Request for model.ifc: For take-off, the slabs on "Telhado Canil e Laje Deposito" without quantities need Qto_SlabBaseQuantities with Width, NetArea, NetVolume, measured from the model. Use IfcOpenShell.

First a look at what the model holds.

```python
import ifcopenshell
import ifcopenshell.util.element
import ifcopenshell.util.unit

model = ifcopenshell.open("model.ifc")
print(model.schema)
for unit_type in ("LENGTHUNIT", "AREAUNIT", "VOLUMEUNIT"):
    print(unit_type, ifcopenshell.util.unit.calculate_unit_scale(model, unit_type))
storey = next(s for s in model.by_type("IfcBuildingStorey") if s.Name == "Telhado Canil e Laje Deposito")
slabs = [e for e in ifcopenshell.util.element.get_decomposition(storey) if e.is_a("IfcSlab")]
for e in sorted(slabs, key=lambda e: e.id()):
    print(e.id(), e.is_a(), e.Name, list(ifcopenshell.util.element.get_psets(e, qtos_only=True)), sep=" | ")
```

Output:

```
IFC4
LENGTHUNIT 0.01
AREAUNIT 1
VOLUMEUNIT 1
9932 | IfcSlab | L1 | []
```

```python
import ifcopenshell
import ifcopenshell.api.pset
import ifcopenshell.geom
import ifcopenshell.util.element
import ifcopenshell.util.shape
import ifcopenshell.util.unit

model = ifcopenshell.open("model.ifc")
unit_scale = ifcopenshell.util.unit.calculate_unit_scale(model)
area_scale = ifcopenshell.util.unit.calculate_unit_scale(model, "AREAUNIT")
volume_scale = ifcopenshell.util.unit.calculate_unit_scale(model, "VOLUMEUNIT")
settings = ifcopenshell.geom.settings()

storey = next(s for s in model.by_type("IfcBuildingStorey") if s.Name == "Telhado Canil e Laje Deposito")
slabs = [e for e in ifcopenshell.util.element.get_decomposition(storey) if e.is_a("IfcSlab")]

for e in sorted(slabs, key=lambda e: e.id()):
    if ifcopenshell.util.element.get_psets(e, qtos_only=True, should_inherit=False):
        continue
    # Geometry comes back in metres, in the element's own axes.
    shape = ifcopenshell.geom.create_shape(settings, e)
    values = {
        "Width": ifcopenshell.util.shape.get_z(shape.geometry) / unit_scale,
        "NetArea": ifcopenshell.util.shape.get_footprint_area(shape.geometry) / area_scale,
        "NetVolume": ifcopenshell.util.shape.get_volume(shape.geometry) / volume_scale,
    }
    qto = ifcopenshell.api.pset.add_qto(model, product=e, name="Qto_SlabBaseQuantities")
    ifcopenshell.api.pset.edit_qto(model, qto=qto, properties=values)
    print(e.id(), {k: round(v, 3) for k, v in values.items()})

model.write("model_rev.ifc")
```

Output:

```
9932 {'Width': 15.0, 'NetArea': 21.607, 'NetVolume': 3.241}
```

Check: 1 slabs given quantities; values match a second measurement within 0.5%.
